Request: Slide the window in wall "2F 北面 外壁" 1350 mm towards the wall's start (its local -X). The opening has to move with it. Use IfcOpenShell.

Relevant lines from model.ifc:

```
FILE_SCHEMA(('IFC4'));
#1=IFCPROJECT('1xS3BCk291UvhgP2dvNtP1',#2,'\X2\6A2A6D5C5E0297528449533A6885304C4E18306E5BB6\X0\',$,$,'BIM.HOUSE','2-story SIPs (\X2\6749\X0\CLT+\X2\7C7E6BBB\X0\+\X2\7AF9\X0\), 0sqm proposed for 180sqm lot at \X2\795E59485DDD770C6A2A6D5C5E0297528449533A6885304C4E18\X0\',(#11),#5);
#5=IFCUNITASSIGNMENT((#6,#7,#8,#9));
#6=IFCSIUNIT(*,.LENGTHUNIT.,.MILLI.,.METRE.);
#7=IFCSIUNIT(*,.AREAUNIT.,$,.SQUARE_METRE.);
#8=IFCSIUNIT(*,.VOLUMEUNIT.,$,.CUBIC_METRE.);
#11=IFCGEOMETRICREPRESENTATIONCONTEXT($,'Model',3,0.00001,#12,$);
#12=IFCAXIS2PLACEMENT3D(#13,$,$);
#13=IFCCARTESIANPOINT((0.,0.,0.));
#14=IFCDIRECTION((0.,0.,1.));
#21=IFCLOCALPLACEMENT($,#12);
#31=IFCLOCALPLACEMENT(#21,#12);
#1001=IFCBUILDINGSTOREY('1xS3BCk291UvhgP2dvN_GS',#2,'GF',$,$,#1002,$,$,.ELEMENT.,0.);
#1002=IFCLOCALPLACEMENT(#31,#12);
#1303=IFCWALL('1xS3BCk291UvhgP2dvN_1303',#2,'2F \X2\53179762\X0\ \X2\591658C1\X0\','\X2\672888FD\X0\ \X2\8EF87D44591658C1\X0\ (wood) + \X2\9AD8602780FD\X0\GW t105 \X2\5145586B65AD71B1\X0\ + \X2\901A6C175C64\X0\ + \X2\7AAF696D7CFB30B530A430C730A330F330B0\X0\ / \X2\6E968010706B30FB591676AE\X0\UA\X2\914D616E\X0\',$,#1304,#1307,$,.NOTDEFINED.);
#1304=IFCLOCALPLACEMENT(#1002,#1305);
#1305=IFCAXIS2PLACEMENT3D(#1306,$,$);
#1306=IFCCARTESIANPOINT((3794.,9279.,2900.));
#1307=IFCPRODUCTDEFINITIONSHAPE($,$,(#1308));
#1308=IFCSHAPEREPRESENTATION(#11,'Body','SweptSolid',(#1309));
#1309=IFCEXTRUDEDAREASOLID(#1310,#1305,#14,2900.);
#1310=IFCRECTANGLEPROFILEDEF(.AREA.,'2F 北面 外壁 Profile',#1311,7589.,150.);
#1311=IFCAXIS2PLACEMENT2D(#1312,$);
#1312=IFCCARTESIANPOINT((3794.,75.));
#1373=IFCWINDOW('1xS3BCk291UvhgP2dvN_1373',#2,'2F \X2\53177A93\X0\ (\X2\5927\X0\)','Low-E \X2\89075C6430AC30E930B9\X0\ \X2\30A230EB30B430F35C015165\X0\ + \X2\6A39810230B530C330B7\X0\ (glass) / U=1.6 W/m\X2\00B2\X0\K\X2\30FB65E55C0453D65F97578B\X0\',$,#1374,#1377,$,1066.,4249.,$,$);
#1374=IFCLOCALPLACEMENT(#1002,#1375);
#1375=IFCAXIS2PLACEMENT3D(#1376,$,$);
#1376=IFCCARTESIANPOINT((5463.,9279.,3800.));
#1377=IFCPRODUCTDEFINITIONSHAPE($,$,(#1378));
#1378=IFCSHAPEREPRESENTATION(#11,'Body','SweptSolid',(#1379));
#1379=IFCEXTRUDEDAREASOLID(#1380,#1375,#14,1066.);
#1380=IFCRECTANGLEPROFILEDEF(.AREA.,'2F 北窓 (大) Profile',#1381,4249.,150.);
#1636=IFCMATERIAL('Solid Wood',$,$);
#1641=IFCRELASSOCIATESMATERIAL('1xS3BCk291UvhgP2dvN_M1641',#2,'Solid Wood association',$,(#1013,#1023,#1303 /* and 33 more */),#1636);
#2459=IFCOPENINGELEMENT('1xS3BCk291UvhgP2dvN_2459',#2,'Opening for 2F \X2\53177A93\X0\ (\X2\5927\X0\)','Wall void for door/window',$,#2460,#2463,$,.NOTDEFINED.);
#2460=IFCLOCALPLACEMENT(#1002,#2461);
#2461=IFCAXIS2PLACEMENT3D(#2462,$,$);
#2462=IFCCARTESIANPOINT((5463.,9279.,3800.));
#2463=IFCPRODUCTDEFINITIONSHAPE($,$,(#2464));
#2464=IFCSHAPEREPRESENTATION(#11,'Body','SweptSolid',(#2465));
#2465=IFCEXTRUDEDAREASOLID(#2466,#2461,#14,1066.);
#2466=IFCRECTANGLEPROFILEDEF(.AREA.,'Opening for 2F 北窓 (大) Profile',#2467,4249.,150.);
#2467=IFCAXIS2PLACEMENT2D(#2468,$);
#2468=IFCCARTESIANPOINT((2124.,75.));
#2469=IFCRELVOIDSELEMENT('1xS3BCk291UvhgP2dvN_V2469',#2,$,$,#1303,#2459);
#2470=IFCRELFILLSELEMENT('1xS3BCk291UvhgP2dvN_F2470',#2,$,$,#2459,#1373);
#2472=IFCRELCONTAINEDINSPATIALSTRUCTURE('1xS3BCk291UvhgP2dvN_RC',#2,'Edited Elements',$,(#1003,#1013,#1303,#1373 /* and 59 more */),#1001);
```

```python
import ifcopenshell
import ifcopenshell.api.geometry
import ifcopenshell.util.placement

model = ifcopenshell.open("model.ifc")

window = model.by_id(1373)
opening = window.FillsVoids[0].RelatingOpeningElement
wall = opening.VoidsElements[0].RelatingBuildingElement

wall_matrix = ifcopenshell.util.placement.get_local_placement(wall.ObjectPlacement)
shift = wall_matrix[:3, 0] * -1350.0
before = ifcopenshell.util.placement.get_local_placement(window.ObjectPlacement)[:3, 3].copy()

# The window is not placed relative to its opening, so move both.
for product in (opening, window):
    matrix = ifcopenshell.util.placement.get_local_placement(product.ObjectPlacement)
    matrix[:3, 3] += shift
    ifcopenshell.api.geometry.edit_object_placement(model, product=product, matrix=matrix, is_si=False)

after = ifcopenshell.util.placement.get_local_placement(window.ObjectPlacement)[:3, 3]
print("window moved by", (after - before).round(3) + 0.0)

model.write("model_edited.ifc")
```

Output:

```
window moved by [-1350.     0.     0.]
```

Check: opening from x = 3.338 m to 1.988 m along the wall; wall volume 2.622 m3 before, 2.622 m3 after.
